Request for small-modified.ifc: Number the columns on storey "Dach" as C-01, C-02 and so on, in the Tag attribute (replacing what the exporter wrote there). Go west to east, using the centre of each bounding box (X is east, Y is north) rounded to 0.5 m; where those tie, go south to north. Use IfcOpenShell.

First a look at what the model holds.

```python
import ifcopenshell
import ifcopenshell.util.element
import ifcopenshell.util.placement

model = ifcopenshell.open("small-modified.ifc")
print(model.schema)
storey = next(s for s in model.by_type("IfcBuildingStorey") if s.Name == "Dach")
columns = [e for e in ifcopenshell.util.element.get_decomposition(storey) if e.is_a("IfcColumn")]
for e in sorted(columns, key=lambda e: e.id()):
    origin = ifcopenshell.util.placement.get_local_placement(e.ObjectPlacement)[:3, 3]
    print(e.id(), e.Tag, e.Name, origin.round(2) + 0.0, sep=" | ")
```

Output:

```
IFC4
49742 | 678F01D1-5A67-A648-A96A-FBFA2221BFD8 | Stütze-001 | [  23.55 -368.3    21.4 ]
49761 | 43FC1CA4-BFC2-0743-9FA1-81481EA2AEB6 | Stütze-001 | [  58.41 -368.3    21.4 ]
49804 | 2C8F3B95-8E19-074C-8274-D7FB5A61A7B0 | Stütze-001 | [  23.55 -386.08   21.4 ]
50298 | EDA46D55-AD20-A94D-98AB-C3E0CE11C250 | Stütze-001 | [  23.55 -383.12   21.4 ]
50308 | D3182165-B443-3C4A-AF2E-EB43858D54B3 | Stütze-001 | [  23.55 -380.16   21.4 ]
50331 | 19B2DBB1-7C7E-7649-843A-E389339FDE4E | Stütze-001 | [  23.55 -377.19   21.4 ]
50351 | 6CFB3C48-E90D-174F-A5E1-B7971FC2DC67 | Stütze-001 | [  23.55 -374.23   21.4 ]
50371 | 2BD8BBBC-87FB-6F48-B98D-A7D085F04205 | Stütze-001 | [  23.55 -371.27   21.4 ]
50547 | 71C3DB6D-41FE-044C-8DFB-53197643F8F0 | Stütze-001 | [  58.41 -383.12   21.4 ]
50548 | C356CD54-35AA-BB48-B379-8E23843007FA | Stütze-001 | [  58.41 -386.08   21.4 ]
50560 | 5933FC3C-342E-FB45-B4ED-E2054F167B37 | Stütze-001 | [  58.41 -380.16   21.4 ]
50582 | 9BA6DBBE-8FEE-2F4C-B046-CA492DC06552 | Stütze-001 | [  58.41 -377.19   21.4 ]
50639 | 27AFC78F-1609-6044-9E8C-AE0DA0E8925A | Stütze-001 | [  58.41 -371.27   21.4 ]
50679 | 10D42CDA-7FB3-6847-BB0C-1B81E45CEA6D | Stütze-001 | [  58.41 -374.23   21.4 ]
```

```python
import ifcopenshell
import ifcopenshell.geom
import ifcopenshell.util.element
import ifcopenshell.util.shape

model = ifcopenshell.open("small-modified.ifc")
settings = ifcopenshell.geom.settings()
settings.set("use-world-coords", True)


def centre(element):
    shape = ifcopenshell.geom.create_shape(settings, element)
    return ifcopenshell.util.shape.get_bbox_centroid(shape.geometry)


storey = next(s for s in model.by_type("IfcBuildingStorey") if s.Name == "Dach")
columns = [e for e in ifcopenshell.util.element.get_decomposition(storey) if e.is_a("IfcColumn")]

# Insertion points can sit at a corner or the storey origin, so sort by the geometry (in metres).
centres = {e: centre(e) for e in columns}
columns.sort(key=lambda e: (round(centres[e][0] / 0.5), centres[e][1]))

for i, e in enumerate(columns, start=1):
    number = f"C-{i:02d}"
    e.Tag = number
    print(e.id(), number)

model.write("small-modified_v2.ifc")
```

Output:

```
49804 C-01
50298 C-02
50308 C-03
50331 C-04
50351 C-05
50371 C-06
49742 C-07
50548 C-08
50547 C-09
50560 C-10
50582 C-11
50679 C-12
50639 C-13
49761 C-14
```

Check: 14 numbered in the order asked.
